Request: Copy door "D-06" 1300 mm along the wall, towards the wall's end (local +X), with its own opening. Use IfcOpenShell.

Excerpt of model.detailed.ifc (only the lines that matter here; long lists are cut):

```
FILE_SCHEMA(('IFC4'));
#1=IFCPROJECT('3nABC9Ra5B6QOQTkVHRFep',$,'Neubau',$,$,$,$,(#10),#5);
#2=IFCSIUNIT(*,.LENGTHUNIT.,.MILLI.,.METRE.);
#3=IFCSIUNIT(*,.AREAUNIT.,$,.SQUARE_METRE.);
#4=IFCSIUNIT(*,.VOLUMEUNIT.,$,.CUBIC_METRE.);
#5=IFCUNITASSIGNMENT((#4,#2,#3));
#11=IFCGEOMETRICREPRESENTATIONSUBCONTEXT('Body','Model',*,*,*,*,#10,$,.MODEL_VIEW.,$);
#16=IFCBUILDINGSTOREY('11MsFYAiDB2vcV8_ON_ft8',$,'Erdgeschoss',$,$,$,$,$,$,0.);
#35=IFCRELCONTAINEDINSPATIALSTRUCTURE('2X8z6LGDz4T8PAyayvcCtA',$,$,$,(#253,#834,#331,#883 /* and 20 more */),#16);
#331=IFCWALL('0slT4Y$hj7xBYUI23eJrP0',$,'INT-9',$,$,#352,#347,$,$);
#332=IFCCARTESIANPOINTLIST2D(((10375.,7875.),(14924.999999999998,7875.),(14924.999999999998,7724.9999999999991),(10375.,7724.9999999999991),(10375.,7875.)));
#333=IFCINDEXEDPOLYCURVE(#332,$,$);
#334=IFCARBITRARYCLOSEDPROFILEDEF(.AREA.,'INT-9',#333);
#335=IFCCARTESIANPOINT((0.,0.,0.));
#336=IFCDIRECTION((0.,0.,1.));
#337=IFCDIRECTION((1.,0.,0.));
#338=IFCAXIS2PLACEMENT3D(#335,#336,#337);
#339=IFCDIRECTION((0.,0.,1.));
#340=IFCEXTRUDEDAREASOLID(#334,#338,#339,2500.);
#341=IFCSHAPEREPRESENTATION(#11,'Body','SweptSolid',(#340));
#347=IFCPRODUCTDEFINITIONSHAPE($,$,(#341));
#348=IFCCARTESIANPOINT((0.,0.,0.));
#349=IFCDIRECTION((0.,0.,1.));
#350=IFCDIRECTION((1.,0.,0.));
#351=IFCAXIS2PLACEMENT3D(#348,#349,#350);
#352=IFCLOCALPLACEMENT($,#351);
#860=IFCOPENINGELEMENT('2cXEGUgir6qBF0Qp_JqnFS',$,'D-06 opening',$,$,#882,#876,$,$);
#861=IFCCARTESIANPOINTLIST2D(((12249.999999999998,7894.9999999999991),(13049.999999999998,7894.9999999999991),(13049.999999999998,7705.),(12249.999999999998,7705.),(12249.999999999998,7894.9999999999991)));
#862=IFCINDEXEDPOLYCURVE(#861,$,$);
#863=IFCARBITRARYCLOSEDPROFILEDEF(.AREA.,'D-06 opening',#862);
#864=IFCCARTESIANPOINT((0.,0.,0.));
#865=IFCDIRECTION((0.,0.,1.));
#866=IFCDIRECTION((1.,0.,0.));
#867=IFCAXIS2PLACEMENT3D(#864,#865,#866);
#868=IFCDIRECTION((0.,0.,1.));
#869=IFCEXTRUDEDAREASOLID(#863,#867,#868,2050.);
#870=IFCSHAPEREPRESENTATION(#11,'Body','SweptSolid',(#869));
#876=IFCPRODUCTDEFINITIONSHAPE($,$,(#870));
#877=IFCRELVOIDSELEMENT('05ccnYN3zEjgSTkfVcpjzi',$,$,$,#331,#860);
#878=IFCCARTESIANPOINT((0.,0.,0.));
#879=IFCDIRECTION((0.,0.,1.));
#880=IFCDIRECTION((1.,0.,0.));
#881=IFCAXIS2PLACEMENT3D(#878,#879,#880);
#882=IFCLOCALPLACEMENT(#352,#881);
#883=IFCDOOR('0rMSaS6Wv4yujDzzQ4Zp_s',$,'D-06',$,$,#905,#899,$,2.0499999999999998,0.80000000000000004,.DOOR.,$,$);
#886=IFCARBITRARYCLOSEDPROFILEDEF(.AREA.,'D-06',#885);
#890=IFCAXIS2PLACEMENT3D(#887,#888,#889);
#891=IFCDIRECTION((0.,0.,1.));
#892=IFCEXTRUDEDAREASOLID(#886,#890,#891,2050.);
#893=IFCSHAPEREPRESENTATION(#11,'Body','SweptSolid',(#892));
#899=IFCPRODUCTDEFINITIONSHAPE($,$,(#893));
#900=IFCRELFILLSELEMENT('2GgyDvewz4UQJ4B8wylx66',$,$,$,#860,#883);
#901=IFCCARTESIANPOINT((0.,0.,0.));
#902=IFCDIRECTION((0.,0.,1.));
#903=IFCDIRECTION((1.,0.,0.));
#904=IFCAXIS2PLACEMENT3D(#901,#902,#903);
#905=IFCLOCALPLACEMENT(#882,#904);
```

```python
import ifcopenshell
import ifcopenshell.api.feature
import ifcopenshell.api.geometry
import ifcopenshell.api.root
import ifcopenshell.geom
import ifcopenshell.util.element
import ifcopenshell.util.placement
import ifcopenshell.util.shape
import ifcopenshell.util.unit

model = ifcopenshell.open("model.detailed.ifc")
unit_scale = ifcopenshell.util.unit.calculate_unit_scale(model)
settings = ifcopenshell.geom.settings()


def volume(element):
    """Net volume in cubic metres, openings subtracted."""
    shape = ifcopenshell.geom.create_shape(settings, element)
    return ifcopenshell.util.shape.get_volume(shape.geometry)


door = model.by_guid("0rMSaS6Wv4yujDzzQ4Zp_s")
opening = door.FillsVoids[0].RelatingOpeningElement
wall = opening.VoidsElements[0].RelatingBuildingElement
before = volume(wall)
shift = ifcopenshell.util.placement.get_local_placement(wall.ObjectPlacement)[:3, 0] * 1.3 / unit_scale

# copy_class copies the void relationship, type, container and properties, but no geometry.
new_opening = ifcopenshell.api.root.copy_class(model, product=opening)
new_opening.Representation = ifcopenshell.util.element.copy_deep(
    model, opening.Representation, exclude=["IfcGeometricRepresentationContext", "IfcRepresentationMap"]
)
new_door = ifcopenshell.api.root.copy_class(model, product=door)
new_door.Representation = ifcopenshell.util.element.copy_deep(
    model, door.Representation, exclude=["IfcGeometricRepresentationContext", "IfcRepresentationMap"]
)
ifcopenshell.api.feature.add_filling(model, opening=new_opening, element=new_door)

for old, new in ((opening, new_opening), (door, new_door)):
    matrix = ifcopenshell.util.placement.get_local_placement(old.ObjectPlacement)
    matrix[:3, 3] += shift
    ifcopenshell.api.geometry.edit_object_placement(model, product=new, matrix=matrix, is_si=False)

after = volume(wall)

print(f"wall volume {before:.3f} -> {after:.3f} m3")

model.write("model.detailed_edited.ifc")
```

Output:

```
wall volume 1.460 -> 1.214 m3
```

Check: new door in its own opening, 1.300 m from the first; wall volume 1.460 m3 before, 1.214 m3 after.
